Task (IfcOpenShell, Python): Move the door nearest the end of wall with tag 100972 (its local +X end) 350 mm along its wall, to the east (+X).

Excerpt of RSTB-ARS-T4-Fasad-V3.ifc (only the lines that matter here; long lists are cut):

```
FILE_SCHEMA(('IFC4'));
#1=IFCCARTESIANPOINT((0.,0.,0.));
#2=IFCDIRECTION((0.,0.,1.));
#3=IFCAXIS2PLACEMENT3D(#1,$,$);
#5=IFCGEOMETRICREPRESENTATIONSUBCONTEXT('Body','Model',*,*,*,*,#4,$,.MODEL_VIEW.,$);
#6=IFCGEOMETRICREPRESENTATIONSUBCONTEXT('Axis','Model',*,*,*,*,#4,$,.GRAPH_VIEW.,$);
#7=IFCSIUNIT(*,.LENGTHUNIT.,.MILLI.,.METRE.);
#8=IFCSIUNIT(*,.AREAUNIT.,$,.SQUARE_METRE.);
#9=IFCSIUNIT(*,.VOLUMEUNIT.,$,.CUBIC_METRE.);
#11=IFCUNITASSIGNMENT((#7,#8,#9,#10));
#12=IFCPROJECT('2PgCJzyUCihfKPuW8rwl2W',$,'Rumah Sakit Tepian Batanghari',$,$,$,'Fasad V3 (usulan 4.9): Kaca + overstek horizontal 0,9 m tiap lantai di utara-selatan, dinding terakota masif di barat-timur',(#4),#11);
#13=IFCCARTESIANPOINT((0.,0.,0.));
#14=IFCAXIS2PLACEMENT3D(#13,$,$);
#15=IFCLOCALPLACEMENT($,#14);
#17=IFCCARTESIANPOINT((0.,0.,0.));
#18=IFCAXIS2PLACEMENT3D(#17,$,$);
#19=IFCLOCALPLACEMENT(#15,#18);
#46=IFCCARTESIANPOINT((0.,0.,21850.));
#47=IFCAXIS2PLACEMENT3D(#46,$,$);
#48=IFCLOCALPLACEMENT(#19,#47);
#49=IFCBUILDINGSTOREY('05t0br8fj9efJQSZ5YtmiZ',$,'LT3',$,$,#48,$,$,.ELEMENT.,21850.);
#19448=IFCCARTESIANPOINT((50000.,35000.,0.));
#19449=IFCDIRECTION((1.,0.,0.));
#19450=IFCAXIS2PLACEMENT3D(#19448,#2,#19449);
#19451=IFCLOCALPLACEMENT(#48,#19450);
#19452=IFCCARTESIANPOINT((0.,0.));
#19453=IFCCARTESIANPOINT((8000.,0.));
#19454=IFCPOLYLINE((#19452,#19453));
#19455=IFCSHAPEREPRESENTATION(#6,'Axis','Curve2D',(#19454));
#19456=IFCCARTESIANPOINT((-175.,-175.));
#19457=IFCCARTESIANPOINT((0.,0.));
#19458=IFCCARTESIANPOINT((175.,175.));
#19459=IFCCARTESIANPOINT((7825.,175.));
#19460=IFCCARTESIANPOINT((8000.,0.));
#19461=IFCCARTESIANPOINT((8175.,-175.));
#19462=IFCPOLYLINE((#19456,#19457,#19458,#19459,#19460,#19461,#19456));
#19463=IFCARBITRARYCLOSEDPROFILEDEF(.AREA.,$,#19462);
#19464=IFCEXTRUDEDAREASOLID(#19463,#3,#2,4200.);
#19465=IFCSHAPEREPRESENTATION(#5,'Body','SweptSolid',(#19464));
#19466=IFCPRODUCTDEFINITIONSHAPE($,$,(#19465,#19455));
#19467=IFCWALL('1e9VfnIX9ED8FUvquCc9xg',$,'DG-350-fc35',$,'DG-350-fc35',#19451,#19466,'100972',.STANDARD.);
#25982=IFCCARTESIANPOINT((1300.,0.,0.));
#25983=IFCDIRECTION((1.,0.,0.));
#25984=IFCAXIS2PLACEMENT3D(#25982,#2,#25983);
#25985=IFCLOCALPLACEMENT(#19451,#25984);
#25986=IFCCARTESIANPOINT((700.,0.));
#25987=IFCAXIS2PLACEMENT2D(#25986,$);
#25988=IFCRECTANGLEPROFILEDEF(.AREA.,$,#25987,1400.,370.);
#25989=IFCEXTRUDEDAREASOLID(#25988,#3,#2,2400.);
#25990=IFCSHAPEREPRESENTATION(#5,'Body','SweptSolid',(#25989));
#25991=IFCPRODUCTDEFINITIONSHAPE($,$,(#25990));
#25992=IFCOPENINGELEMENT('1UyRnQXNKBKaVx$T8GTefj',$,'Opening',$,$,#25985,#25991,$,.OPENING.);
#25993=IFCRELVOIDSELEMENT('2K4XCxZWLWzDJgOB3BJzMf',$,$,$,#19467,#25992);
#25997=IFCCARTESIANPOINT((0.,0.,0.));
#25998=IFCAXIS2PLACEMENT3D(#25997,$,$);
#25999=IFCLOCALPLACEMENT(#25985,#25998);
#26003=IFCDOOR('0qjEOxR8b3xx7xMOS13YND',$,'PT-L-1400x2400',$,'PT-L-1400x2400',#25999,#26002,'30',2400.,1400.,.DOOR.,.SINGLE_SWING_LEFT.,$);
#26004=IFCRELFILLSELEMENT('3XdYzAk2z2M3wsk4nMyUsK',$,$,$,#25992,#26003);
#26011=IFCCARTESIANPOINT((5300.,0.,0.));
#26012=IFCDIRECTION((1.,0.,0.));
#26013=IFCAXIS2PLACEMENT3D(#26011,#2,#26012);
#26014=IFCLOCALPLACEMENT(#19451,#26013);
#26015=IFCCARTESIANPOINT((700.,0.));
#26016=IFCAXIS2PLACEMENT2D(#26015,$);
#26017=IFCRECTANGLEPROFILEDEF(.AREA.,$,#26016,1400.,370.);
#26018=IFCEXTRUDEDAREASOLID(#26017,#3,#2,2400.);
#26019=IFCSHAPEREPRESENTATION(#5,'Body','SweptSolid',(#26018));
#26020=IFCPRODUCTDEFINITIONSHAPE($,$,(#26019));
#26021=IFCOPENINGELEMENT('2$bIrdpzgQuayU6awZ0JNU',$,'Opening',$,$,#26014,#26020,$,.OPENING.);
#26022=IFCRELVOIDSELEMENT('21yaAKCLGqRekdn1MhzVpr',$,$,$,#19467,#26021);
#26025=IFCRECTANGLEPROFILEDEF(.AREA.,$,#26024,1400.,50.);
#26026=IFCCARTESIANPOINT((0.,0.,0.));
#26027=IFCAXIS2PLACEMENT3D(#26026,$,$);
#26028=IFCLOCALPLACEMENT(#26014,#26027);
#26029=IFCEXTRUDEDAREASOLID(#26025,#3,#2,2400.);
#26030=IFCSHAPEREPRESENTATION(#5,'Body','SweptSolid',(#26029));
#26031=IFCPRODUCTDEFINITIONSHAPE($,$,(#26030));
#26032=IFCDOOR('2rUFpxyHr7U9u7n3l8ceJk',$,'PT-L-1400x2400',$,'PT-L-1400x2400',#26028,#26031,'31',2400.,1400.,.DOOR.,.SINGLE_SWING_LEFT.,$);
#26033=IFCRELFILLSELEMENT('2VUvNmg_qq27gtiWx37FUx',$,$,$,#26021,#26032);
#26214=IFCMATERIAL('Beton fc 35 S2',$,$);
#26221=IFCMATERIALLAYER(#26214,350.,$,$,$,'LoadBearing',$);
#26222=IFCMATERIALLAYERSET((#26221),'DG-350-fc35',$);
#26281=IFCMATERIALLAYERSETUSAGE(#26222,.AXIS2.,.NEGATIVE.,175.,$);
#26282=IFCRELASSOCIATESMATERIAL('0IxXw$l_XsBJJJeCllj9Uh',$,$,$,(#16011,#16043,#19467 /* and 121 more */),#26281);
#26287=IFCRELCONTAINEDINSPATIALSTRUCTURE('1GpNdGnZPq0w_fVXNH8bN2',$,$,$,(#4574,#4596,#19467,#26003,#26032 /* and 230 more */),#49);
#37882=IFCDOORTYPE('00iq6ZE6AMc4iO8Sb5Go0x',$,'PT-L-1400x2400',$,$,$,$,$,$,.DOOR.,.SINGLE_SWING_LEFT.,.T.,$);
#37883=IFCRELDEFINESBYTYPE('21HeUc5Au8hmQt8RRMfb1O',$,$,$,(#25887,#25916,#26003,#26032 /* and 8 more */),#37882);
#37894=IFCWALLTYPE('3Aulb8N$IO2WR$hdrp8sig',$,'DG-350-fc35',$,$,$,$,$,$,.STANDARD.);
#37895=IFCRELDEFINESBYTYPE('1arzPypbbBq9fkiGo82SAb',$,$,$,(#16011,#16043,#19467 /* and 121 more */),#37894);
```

```python
import ifcopenshell
import ifcopenshell.api.geometry
import ifcopenshell.util.placement
import ifcopenshell.util.unit

model = ifcopenshell.open("RSTB-ARS-T4-Fasad-V3.ifc")
unit_scale = ifcopenshell.util.unit.calculate_unit_scale(model)

door = model.by_guid("2rUFpxyHr7U9u7n3l8ceJk")
opening = door.FillsVoids[0].RelatingOpeningElement
wall = opening.VoidsElements[0].RelatingBuildingElement

wall_matrix = ifcopenshell.util.placement.get_local_placement(wall.ObjectPlacement)
shift = wall_matrix[:3, 0] * 0.35 / unit_scale
before = ifcopenshell.util.placement.get_local_placement(door.ObjectPlacement)[:3, 3].copy()

# The door is placed relative to its opening, so it follows when the opening moves.
matrix = ifcopenshell.util.placement.get_local_placement(opening.ObjectPlacement)
matrix[:3, 3] += shift
ifcopenshell.api.geometry.edit_object_placement(
    model, product=opening, matrix=matrix, is_si=False, should_transform_children=True
)

after = ifcopenshell.util.placement.get_local_placement(door.ObjectPlacement)[:3, 3]
print("door moved by", (after - before).round(3) + 0.0)

model.write("RSTB-ARS-T4-Fasad-V3-out.ifc")
```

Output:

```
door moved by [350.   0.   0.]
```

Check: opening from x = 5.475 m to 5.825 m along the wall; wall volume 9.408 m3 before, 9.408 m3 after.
